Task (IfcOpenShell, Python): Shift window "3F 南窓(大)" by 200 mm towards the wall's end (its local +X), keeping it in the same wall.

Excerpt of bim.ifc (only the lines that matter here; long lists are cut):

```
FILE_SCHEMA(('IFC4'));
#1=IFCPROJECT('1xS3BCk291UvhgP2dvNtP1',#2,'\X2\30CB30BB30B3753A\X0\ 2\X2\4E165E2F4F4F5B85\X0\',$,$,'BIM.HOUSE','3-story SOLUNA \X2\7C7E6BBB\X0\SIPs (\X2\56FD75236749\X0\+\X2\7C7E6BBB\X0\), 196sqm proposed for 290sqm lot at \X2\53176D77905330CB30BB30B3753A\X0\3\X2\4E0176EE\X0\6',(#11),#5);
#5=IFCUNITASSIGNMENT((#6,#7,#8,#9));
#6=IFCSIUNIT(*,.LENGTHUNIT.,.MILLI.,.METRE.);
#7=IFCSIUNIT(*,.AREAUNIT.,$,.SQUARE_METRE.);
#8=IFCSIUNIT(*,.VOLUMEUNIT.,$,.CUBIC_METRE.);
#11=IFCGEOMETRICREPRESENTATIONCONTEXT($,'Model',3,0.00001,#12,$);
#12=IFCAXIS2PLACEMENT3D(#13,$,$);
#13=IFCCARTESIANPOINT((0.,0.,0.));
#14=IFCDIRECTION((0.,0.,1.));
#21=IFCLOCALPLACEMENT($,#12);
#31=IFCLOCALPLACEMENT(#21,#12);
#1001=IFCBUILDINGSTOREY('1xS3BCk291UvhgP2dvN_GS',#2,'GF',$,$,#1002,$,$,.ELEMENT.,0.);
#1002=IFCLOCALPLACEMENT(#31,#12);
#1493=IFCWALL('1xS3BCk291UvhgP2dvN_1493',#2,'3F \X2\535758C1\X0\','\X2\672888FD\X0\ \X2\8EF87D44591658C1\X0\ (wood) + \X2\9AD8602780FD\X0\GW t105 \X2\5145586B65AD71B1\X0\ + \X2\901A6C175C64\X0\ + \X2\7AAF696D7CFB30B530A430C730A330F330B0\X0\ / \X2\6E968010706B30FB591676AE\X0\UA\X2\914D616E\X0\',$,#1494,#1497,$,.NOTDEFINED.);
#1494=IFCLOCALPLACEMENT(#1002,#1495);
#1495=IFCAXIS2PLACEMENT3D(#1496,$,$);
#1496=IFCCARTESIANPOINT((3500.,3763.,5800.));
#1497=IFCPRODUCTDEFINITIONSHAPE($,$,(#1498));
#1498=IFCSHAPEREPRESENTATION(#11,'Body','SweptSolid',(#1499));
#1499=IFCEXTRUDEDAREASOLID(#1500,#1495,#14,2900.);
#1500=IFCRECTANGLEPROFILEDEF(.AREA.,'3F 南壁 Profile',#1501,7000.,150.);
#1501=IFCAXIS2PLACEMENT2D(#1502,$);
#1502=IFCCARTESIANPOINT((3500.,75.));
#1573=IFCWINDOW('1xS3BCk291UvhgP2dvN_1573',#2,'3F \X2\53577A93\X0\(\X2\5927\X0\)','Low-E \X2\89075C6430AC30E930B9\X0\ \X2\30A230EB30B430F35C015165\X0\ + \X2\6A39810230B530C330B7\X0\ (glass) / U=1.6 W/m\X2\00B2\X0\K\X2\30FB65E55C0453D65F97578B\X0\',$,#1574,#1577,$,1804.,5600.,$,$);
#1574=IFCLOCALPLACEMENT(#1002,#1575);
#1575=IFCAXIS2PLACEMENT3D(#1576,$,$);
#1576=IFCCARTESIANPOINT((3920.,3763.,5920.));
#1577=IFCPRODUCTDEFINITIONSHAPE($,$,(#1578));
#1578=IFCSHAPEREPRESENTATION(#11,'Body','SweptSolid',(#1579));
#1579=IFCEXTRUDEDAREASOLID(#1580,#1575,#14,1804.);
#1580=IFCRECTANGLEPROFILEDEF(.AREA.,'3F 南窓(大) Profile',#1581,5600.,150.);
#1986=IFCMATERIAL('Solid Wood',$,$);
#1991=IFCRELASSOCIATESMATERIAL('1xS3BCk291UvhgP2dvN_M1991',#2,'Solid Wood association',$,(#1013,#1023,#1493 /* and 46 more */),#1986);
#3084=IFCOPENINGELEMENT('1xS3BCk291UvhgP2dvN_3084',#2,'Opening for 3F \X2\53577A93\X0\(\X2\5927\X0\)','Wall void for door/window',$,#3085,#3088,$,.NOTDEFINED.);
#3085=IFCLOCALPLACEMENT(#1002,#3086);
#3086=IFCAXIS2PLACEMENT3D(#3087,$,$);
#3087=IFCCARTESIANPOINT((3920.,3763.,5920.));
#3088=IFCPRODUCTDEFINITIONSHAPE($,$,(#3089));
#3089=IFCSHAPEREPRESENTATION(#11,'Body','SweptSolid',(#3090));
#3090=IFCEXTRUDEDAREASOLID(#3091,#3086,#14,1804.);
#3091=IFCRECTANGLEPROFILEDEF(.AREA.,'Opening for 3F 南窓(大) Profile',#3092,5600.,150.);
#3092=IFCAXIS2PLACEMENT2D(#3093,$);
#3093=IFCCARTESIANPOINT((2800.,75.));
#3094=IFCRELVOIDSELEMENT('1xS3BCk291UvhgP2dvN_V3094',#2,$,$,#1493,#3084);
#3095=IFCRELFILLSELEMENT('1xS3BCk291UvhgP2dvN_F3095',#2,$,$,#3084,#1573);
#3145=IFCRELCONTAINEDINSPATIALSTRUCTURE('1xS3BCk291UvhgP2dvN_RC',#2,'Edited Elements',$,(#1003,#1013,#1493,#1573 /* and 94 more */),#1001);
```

```python
import ifcopenshell
import ifcopenshell.api.geometry
import ifcopenshell.util.placement
import ifcopenshell.util.unit

model = ifcopenshell.open("bim.ifc")
unit_scale = ifcopenshell.util.unit.calculate_unit_scale(model)

window = model.by_guid("1xS3BCk291UvhgP2dvN_1573")
opening = window.FillsVoids[0].RelatingOpeningElement
wall = opening.VoidsElements[0].RelatingBuildingElement

wall_matrix = ifcopenshell.util.placement.get_local_placement(wall.ObjectPlacement)
shift = wall_matrix[:3, 0] * 0.2 / unit_scale
before = ifcopenshell.util.placement.get_local_placement(window.ObjectPlacement)[:3, 3].copy()

# The window is not placed relative to its opening, so move both.
for product in (opening, window):
    matrix = ifcopenshell.util.placement.get_local_placement(product.ObjectPlacement)
    matrix[:3, 3] += shift
    ifcopenshell.api.geometry.edit_object_placement(model, product=product, matrix=matrix, is_si=False)

after = ifcopenshell.util.placement.get_local_placement(window.ObjectPlacement)[:3, 3]
print("window moved by", (after - before).round(3) + 0.0)

model.write("bim_rev.ifc")
```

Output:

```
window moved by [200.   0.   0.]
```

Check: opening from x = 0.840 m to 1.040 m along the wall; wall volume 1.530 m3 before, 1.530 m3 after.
